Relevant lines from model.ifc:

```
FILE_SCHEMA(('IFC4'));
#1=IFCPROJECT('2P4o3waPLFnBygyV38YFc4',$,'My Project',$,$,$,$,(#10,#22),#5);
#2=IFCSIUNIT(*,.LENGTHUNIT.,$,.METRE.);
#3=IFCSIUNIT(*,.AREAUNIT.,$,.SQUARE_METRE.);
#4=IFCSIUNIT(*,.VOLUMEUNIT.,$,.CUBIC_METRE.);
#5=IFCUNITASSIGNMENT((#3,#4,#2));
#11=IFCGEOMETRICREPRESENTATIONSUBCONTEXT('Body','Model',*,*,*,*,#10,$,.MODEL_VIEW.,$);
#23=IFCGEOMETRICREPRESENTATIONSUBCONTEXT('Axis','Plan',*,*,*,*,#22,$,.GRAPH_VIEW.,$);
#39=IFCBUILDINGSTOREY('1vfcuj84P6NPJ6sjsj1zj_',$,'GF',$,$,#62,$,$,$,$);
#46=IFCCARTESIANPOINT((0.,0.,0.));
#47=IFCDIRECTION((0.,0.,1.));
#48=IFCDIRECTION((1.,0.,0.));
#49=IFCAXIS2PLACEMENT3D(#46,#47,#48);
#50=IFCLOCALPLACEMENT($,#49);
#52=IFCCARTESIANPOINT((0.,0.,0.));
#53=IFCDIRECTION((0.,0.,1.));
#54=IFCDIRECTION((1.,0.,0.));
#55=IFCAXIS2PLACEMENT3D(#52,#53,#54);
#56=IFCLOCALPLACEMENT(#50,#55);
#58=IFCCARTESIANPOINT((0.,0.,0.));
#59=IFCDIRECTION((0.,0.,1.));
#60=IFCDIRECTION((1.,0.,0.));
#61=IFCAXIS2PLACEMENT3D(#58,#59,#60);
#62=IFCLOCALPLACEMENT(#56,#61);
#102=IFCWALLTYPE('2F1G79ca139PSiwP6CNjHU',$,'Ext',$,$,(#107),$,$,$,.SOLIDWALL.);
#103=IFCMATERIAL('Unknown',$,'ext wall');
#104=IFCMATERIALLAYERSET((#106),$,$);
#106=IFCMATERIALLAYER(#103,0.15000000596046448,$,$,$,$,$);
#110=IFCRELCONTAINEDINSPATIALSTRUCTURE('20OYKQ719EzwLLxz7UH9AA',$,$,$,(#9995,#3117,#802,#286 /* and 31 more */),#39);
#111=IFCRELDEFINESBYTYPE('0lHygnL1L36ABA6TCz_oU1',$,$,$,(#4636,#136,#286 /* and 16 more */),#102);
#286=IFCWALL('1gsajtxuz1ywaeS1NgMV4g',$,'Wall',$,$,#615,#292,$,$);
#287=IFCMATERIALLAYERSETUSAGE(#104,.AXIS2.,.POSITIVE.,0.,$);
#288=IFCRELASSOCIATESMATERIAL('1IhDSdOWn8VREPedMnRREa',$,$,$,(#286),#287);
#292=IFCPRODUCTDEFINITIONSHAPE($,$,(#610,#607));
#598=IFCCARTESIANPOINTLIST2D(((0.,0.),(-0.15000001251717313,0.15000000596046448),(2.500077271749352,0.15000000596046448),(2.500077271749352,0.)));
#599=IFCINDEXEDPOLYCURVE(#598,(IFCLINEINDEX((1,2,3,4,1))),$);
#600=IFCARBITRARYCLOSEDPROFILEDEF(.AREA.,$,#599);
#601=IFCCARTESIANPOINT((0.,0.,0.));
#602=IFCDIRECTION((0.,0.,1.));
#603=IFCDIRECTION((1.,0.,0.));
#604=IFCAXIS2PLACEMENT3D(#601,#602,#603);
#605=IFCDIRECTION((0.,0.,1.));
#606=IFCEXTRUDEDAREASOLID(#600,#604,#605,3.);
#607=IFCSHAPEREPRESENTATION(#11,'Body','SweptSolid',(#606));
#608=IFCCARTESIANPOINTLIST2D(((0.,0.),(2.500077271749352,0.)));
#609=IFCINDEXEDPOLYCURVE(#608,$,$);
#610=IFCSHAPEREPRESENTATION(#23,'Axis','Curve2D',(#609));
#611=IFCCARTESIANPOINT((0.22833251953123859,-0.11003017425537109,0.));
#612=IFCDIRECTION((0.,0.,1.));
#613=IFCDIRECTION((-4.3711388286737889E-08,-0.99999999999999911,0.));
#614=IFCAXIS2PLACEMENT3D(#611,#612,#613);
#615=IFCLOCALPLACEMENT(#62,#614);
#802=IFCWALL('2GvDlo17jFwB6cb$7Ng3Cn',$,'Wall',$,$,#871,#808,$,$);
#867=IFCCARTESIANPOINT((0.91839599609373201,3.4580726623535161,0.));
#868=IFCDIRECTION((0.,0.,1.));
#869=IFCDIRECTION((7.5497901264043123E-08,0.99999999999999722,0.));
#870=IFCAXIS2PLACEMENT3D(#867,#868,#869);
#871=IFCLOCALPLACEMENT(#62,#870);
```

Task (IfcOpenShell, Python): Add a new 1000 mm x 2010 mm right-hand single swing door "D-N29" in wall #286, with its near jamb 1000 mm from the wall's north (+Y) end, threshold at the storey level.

```python
import numpy as np
import ifcopenshell
import ifcopenshell.api.feature
import ifcopenshell.api.geometry
import ifcopenshell.api.root
import ifcopenshell.api.spatial
import ifcopenshell.geom
import ifcopenshell.util.element
import ifcopenshell.util.placement
import ifcopenshell.util.representation
import ifcopenshell.util.shape
import ifcopenshell.util.unit

model = ifcopenshell.open("model.ifc")
unit_scale = ifcopenshell.util.unit.calculate_unit_scale(model)
settings = ifcopenshell.geom.settings()


def volume(element):
    """Net volume in cubic metres, openings subtracted."""
    shape = ifcopenshell.geom.create_shape(settings, element)
    return ifcopenshell.util.shape.get_volume(shape.geometry)


wall = model.by_guid("1gsajtxuz1ywaeS1NgMV4g")
storey = ifcopenshell.util.element.get_container(wall, ifc_class="IfcBuildingStorey")
context = ifcopenshell.util.representation.get_context(model, "Model", "Body", "MODEL_VIEW")
before = volume(wall)

width, height, from_end, sill = 1, 2.01, 1, 0.0  # metres

# The wall runs along its own X axis, and the end named is its -X end.
wall_shape = ifcopenshell.geom.create_shape(settings, wall)
x, y, z = ifcopenshell.util.shape.get_vertices(wall_shape.geometry).T
start = x.min() + from_end
face, thickness = float(y.min()), float(y.max() - y.min())
wall_matrix = ifcopenshell.util.placement.get_local_placement(wall.ObjectPlacement)
level = ifcopenshell.util.placement.get_local_placement(storey.ObjectPlacement)[2, 3]


def in_wall(x, y):
    """Placement at x, y metres in the wall's axes, at sill height."""
    matrix = wall_matrix.copy()
    matrix[:, 3] = wall_matrix @ np.array([x / unit_scale, y / unit_scale, 0.0, 1.0])
    matrix[2, 3] = level + sill / unit_scale
    return matrix


# Opening: a box that overshoots both wall faces by 50 mm.
opening = ifcopenshell.api.root.create_entity(model, ifc_class="IfcOpeningElement", predefined_type="OPENING")
box = ifcopenshell.api.geometry.add_wall_representation(
    model, context=context, length=width, height=height, thickness=thickness + 0.1
)
ifcopenshell.api.geometry.assign_representation(model, product=opening, representation=box)
ifcopenshell.api.geometry.edit_object_placement(model, product=opening, matrix=in_wall(start, face - 0.05), is_si=False)
ifcopenshell.api.feature.add_feature(model, feature=opening, element=wall)

door = ifcopenshell.api.root.create_entity(model, ifc_class="IfcDoor", name="D-N29", predefined_type="DOOR")
door.OverallWidth, door.OverallHeight = width / unit_scale, height / unit_scale
door.OperationType = "SINGLE_SWING_RIGHT"
body = ifcopenshell.api.geometry.add_door_representation(
    model,
    context=context,
    overall_width=door.OverallWidth,
    overall_height=door.OverallHeight,
    operation_type="SINGLE_SWING_RIGHT",
    lining_properties={"LiningDepth": thickness / unit_scale, "ThresholdDepth": thickness / unit_scale},
)
ifcopenshell.api.geometry.assign_representation(model, product=door, representation=body)
ifcopenshell.api.spatial.assign_container(model, products=[door], relating_structure=storey)
ifcopenshell.api.feature.add_filling(model, opening=opening, element=door)

# The lining spans the wall, so the door starts at the wall face.
ifcopenshell.api.geometry.edit_object_placement(model, product=door, matrix=in_wall(start, face), is_si=False)

after = volume(wall)

print(f"wall volume {before:.3f} -> {after:.3f} m3")

model.write("model_updated.ifc")
```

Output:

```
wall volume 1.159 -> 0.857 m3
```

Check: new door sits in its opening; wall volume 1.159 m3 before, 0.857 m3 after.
